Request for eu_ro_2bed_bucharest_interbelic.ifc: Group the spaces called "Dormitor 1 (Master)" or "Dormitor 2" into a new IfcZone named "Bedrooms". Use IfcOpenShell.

First a look at what the model holds.

```python
import ifcopenshell

model = ifcopenshell.open("eu_ro_2bed_bucharest_interbelic.ifc")
print(model.schema)
seen = {}
for space in model.by_type("IfcSpace"):
    seen[space.LongName] = seen.get(space.LongName, 0) + 1
for name, count in sorted(seen.items(), key=str):
    print(count, "x", name)
print("zones:", [z.Name for z in model.by_type("IfcZone")][:20])
```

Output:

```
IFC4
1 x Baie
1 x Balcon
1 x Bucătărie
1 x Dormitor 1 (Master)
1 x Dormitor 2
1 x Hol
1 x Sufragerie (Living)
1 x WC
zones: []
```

```python
import ifcopenshell
import ifcopenshell.api.group
import ifcopenshell.api.root

model = ifcopenshell.open("eu_ro_2bed_bucharest_interbelic.ifc")

names = {"Dormitor 1 (Master)", "Dormitor 2"}
spaces = [s for s in model.by_type("IfcSpace") if s.LongName in names]

zone = ifcopenshell.api.root.create_entity(model, ifc_class="IfcZone", name="Bedrooms")
ifcopenshell.api.group.assign_group(model, products=spaces, group=zone)
print(len(spaces), "spaces in", zone.Name)

model.write("eu_ro_2bed_bucharest_interbelic_updated.ifc")
```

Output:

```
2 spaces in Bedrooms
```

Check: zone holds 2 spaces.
